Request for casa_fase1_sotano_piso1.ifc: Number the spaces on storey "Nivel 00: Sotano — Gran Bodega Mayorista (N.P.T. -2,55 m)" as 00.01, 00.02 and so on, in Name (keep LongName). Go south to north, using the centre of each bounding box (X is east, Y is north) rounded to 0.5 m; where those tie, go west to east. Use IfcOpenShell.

First a look at what the model holds.

```python
import ifcopenshell
import ifcopenshell.util.element
import ifcopenshell.util.placement

model = ifcopenshell.open("casa_fase1_sotano_piso1.ifc")
print(model.schema)
storey = next(s for s in model.by_type("IfcBuildingStorey") if s.Name == "Nivel 00: Sotano — Gran Bodega Mayorista (N.P.T. -2,55 m)")
spaces = [e for e in ifcopenshell.util.element.get_decomposition(storey) if e.is_a("IfcSpace")]
for e in sorted(spaces, key=lambda e: e.id()):
    origin = ifcopenshell.util.placement.get_local_placement(e.ObjectPlacement)[:3, 3]
    print(e.id(), e.Name, e.LongName, origin.round(2) + 0.0, sep=" | ")
```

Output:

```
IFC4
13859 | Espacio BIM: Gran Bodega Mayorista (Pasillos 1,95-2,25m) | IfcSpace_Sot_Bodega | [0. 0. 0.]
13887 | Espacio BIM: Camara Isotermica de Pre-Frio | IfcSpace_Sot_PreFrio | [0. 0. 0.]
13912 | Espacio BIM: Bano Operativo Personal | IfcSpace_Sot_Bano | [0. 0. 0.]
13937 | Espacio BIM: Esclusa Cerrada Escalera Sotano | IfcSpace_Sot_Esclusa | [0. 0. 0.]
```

```python
import ifcopenshell
import ifcopenshell.geom
import ifcopenshell.util.element
import ifcopenshell.util.shape

model = ifcopenshell.open("casa_fase1_sotano_piso1.ifc")
settings = ifcopenshell.geom.settings()
settings.set("use-world-coords", True)


def centre(element):
    shape = ifcopenshell.geom.create_shape(settings, element)
    return ifcopenshell.util.shape.get_bbox_centroid(shape.geometry)


storey = next(s for s in model.by_type("IfcBuildingStorey") if s.Name == "Nivel 00: Sotano — Gran Bodega Mayorista (N.P.T. -2,55 m)")
spaces = [e for e in ifcopenshell.util.element.get_decomposition(storey) if e.is_a("IfcSpace")]

# Insertion points can sit at a corner or the storey origin, so sort by the geometry (in metres).
centres = {e: centre(e) for e in spaces}
spaces.sort(key=lambda e: (round(centres[e][1] / 0.5), centres[e][0]))

for i, e in enumerate(spaces, start=1):
    number = f"00.{i:02d}"
    e.Name = number
    print(e.id(), number)

model.write("casa_fase1_sotano_piso1_updated.ifc")
```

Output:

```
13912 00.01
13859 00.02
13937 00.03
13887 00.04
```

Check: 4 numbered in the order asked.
